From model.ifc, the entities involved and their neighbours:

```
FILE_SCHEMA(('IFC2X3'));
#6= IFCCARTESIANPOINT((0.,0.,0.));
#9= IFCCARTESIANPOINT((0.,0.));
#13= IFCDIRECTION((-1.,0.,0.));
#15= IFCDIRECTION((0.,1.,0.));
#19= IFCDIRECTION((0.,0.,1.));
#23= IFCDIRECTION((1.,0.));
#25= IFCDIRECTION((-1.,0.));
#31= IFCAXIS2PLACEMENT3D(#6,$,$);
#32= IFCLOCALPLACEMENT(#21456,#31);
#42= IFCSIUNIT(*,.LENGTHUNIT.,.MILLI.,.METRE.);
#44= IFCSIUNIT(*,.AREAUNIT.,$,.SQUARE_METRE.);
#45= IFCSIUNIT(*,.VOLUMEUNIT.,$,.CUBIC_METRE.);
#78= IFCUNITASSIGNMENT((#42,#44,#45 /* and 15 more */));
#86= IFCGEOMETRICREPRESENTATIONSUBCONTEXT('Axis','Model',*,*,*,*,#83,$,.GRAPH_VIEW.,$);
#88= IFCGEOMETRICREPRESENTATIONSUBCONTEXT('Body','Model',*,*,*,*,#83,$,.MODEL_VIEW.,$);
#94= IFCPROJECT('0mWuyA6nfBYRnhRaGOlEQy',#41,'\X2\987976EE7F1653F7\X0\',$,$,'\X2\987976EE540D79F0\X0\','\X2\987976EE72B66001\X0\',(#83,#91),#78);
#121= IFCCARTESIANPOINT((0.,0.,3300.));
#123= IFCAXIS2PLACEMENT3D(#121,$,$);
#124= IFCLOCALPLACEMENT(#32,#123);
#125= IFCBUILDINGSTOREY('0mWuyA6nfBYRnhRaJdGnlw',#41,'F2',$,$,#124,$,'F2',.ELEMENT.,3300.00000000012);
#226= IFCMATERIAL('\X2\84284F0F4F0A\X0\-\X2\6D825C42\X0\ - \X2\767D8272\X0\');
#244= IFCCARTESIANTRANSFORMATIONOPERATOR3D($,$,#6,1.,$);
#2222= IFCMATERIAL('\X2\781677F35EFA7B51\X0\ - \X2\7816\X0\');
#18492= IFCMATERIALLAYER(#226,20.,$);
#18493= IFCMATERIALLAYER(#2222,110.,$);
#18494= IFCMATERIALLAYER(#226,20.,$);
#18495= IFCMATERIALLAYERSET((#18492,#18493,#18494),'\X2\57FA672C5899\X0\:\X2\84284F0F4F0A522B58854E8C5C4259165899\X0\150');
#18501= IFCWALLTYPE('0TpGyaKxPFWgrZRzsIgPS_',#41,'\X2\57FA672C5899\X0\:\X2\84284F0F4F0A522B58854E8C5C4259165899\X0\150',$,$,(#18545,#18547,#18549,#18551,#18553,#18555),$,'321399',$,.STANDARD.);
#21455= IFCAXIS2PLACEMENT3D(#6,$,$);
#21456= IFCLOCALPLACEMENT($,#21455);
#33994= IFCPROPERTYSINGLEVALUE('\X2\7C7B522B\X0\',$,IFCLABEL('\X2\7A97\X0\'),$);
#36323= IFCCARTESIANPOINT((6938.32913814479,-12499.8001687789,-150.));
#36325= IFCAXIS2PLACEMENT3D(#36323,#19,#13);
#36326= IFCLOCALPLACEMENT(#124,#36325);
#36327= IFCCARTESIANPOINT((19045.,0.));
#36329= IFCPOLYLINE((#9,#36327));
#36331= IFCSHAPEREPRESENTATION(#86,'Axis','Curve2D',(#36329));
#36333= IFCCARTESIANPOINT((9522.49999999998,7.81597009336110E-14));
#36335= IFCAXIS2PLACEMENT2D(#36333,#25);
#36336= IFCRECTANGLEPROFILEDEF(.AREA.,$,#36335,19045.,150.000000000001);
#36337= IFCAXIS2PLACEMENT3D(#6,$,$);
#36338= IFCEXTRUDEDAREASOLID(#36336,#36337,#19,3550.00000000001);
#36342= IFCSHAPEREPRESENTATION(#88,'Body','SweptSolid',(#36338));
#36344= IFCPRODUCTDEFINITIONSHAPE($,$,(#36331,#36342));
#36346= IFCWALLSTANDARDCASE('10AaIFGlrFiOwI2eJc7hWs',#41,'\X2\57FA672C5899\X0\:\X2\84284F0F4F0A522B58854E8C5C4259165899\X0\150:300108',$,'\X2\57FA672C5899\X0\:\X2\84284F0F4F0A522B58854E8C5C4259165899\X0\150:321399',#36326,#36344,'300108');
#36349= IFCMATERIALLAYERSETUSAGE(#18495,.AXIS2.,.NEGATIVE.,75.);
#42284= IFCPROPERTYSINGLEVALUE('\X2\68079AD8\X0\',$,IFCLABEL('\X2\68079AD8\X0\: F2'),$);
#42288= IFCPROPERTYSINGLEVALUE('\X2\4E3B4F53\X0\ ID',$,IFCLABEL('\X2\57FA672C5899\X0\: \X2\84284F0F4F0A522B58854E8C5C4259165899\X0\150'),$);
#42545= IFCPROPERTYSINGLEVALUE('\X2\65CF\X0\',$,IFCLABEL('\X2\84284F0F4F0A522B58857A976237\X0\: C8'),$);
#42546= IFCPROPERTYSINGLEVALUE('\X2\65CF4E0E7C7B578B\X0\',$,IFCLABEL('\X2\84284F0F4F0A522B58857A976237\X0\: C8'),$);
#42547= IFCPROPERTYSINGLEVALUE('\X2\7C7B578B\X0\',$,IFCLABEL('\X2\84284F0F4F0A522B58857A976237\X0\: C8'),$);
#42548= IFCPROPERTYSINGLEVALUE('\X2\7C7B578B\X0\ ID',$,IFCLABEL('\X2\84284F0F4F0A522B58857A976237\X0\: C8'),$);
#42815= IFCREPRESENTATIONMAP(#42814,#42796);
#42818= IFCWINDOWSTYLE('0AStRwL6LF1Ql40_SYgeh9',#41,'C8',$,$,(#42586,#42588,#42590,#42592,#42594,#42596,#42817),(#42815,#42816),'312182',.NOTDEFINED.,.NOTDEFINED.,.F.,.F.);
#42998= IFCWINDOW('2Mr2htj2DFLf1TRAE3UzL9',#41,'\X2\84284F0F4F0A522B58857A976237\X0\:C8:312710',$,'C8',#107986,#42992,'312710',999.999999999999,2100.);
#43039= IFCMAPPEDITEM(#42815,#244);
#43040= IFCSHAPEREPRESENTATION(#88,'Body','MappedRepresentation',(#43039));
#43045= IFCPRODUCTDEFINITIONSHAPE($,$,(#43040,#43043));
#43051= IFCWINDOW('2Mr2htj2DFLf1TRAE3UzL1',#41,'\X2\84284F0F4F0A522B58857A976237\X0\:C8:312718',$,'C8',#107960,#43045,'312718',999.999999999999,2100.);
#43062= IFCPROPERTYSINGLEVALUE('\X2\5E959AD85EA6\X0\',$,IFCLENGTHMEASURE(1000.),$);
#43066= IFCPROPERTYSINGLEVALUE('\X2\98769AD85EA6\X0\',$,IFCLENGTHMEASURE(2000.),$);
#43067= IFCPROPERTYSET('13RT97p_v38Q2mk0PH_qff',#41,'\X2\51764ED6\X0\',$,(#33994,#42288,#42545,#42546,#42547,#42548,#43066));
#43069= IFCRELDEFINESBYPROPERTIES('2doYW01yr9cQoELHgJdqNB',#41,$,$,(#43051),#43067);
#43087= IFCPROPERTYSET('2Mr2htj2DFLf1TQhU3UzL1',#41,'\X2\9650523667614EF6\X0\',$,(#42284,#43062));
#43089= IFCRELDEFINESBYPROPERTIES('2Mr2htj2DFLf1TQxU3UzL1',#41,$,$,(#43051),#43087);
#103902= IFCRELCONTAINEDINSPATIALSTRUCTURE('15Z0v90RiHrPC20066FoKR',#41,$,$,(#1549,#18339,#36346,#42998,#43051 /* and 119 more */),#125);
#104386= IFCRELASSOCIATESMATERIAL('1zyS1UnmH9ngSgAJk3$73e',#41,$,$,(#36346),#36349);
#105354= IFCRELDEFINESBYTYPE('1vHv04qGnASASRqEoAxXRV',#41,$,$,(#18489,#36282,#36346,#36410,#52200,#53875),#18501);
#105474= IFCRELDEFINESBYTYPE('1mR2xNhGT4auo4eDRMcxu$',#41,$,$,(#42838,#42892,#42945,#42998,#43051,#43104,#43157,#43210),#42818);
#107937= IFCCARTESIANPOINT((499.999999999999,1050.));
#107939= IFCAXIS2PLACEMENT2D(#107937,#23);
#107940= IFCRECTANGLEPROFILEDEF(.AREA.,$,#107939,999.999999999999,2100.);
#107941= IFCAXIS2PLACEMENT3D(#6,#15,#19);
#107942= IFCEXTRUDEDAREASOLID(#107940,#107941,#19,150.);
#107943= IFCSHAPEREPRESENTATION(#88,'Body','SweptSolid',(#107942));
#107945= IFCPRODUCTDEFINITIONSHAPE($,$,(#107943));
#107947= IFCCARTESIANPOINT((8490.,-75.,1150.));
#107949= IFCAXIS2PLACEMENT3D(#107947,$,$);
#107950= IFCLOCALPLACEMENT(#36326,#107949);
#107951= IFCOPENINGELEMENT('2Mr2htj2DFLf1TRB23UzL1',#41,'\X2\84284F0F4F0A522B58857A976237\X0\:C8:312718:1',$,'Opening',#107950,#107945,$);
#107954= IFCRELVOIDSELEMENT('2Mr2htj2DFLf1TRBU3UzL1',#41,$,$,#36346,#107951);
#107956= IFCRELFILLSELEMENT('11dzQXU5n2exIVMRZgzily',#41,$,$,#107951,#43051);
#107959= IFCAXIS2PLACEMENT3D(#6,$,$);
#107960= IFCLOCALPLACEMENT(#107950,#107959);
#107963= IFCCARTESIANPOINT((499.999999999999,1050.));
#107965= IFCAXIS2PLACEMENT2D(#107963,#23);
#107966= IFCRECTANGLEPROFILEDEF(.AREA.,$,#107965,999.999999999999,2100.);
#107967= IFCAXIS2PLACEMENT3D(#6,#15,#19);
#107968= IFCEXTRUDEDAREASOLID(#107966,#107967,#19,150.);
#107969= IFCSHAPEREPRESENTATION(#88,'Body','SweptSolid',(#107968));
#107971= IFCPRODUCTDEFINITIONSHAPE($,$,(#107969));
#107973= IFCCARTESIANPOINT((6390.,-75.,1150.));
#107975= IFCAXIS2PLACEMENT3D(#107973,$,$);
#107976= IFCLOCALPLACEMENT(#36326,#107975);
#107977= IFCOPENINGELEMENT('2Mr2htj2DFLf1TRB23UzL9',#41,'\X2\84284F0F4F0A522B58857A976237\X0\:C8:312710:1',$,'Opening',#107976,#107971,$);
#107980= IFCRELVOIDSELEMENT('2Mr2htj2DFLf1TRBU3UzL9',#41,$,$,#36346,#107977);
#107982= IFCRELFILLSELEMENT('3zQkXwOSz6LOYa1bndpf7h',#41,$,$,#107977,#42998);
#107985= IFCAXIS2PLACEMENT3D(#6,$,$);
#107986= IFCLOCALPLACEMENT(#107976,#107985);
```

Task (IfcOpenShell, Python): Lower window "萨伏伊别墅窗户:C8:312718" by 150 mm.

```python
import numpy as np
import ifcopenshell
import ifcopenshell.api.geometry
import ifcopenshell.api.pset
import ifcopenshell.util.element
import ifcopenshell.util.placement
import ifcopenshell.util.unit

model = ifcopenshell.open("model.ifc")
unit_scale = ifcopenshell.util.unit.calculate_unit_scale(model)

window = model.by_guid("2Mr2htj2DFLf1TRAE3UzL1")
opening = window.FillsVoids[0].RelatingOpeningElement
dz = -150.0

shift = np.array([0.0, 0.0, dz])
# The window is placed relative to its opening, so it follows when the opening moves.
matrix = ifcopenshell.util.placement.get_local_placement(opening.ObjectPlacement)
matrix[:3, 3] += shift
ifcopenshell.api.geometry.edit_object_placement(
    model, product=opening, matrix=matrix, is_si=False, should_transform_children=True
)

# Keep the stored heights in step.
pset = model.by_id(ifcopenshell.util.element.get_pset(window, "其他", should_inherit=False)["id"])
ifcopenshell.api.pset.edit_pset(model, pset=pset, properties={
    "顶高度": model.create_entity("IfcLengthMeasure", ifcopenshell.util.element.get_pset(window, "其他", "顶高度") + dz),
})
pset = model.by_id(ifcopenshell.util.element.get_pset(window, "限制条件", should_inherit=False)["id"])
ifcopenshell.api.pset.edit_pset(model, pset=pset, properties={
    "底高度": model.create_entity("IfcLengthMeasure", ifcopenshell.util.element.get_pset(window, "限制条件", "底高度") + dz),
})

print(f"moved by {dz * unit_scale:+.3f} m")

model.write("model_v2.ifc")
```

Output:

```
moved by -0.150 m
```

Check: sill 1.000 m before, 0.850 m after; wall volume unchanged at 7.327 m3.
